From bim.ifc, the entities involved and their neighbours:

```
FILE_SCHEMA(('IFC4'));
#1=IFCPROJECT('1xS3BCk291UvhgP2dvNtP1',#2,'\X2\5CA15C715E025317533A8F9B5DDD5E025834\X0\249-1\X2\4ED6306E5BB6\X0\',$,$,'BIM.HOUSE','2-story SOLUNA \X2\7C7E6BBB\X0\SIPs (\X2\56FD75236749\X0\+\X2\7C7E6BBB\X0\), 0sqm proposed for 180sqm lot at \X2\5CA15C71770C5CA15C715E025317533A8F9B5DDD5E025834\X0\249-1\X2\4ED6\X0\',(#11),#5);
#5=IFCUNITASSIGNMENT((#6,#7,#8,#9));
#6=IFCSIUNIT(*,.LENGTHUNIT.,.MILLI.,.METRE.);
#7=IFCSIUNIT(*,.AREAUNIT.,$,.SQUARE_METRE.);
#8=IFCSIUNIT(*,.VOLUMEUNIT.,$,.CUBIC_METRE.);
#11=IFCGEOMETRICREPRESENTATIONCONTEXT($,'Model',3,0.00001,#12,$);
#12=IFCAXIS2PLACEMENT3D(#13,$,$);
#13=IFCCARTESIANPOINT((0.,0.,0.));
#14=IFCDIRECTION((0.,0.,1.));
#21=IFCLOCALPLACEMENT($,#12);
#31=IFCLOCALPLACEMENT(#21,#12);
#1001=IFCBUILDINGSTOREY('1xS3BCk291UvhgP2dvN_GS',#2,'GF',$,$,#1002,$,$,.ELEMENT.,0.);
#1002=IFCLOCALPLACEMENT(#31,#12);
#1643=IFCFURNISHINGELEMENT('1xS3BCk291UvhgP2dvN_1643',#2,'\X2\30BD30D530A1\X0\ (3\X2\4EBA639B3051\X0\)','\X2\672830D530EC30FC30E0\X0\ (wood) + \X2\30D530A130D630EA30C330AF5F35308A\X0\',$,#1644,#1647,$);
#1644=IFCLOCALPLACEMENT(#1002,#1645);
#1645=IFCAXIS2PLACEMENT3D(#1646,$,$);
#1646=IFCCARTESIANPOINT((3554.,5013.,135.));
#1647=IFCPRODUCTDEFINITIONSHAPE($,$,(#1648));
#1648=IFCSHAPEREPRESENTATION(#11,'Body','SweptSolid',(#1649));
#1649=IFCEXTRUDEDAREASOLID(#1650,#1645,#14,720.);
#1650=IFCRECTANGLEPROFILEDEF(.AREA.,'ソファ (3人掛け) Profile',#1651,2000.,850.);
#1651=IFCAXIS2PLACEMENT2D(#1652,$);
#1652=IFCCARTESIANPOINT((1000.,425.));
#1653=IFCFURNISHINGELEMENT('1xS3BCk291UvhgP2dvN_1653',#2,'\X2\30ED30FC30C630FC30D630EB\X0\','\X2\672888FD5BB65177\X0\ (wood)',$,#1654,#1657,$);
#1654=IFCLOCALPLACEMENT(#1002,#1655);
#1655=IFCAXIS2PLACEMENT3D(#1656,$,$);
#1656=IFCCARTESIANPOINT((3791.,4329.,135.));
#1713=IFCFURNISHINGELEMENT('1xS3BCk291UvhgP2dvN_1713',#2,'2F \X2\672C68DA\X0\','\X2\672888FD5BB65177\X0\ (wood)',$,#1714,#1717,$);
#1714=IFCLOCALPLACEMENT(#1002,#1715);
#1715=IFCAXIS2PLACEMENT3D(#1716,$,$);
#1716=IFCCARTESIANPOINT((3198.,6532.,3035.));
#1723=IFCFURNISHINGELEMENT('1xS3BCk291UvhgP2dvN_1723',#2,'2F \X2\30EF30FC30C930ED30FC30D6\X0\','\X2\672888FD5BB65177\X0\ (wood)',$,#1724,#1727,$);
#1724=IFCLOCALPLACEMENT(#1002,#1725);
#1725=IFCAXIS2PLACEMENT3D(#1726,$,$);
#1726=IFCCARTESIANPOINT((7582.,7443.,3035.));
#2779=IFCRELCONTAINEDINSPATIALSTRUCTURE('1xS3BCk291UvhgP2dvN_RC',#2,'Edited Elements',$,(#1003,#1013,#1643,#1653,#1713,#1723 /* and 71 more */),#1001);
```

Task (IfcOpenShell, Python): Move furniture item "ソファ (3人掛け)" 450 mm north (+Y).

```python
import ifcopenshell
import ifcopenshell.api.geometry
import ifcopenshell.util.placement

model = ifcopenshell.open("bim.ifc")

item = model.by_guid("1xS3BCk291UvhgP2dvN_1643")
matrix = ifcopenshell.util.placement.get_local_placement(item.ObjectPlacement)
matrix[1, 3] += 450.0
ifcopenshell.api.geometry.edit_object_placement(model, product=item, matrix=matrix, is_si=False)

print(ifcopenshell.util.placement.get_local_placement(item.ObjectPlacement).round(3) + 0.0)

model.write("bim_v2.ifc")
```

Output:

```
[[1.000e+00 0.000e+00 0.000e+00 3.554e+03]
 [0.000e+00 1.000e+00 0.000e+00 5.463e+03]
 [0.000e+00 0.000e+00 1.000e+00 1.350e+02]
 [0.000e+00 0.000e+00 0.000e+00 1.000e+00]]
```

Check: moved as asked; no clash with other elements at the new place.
